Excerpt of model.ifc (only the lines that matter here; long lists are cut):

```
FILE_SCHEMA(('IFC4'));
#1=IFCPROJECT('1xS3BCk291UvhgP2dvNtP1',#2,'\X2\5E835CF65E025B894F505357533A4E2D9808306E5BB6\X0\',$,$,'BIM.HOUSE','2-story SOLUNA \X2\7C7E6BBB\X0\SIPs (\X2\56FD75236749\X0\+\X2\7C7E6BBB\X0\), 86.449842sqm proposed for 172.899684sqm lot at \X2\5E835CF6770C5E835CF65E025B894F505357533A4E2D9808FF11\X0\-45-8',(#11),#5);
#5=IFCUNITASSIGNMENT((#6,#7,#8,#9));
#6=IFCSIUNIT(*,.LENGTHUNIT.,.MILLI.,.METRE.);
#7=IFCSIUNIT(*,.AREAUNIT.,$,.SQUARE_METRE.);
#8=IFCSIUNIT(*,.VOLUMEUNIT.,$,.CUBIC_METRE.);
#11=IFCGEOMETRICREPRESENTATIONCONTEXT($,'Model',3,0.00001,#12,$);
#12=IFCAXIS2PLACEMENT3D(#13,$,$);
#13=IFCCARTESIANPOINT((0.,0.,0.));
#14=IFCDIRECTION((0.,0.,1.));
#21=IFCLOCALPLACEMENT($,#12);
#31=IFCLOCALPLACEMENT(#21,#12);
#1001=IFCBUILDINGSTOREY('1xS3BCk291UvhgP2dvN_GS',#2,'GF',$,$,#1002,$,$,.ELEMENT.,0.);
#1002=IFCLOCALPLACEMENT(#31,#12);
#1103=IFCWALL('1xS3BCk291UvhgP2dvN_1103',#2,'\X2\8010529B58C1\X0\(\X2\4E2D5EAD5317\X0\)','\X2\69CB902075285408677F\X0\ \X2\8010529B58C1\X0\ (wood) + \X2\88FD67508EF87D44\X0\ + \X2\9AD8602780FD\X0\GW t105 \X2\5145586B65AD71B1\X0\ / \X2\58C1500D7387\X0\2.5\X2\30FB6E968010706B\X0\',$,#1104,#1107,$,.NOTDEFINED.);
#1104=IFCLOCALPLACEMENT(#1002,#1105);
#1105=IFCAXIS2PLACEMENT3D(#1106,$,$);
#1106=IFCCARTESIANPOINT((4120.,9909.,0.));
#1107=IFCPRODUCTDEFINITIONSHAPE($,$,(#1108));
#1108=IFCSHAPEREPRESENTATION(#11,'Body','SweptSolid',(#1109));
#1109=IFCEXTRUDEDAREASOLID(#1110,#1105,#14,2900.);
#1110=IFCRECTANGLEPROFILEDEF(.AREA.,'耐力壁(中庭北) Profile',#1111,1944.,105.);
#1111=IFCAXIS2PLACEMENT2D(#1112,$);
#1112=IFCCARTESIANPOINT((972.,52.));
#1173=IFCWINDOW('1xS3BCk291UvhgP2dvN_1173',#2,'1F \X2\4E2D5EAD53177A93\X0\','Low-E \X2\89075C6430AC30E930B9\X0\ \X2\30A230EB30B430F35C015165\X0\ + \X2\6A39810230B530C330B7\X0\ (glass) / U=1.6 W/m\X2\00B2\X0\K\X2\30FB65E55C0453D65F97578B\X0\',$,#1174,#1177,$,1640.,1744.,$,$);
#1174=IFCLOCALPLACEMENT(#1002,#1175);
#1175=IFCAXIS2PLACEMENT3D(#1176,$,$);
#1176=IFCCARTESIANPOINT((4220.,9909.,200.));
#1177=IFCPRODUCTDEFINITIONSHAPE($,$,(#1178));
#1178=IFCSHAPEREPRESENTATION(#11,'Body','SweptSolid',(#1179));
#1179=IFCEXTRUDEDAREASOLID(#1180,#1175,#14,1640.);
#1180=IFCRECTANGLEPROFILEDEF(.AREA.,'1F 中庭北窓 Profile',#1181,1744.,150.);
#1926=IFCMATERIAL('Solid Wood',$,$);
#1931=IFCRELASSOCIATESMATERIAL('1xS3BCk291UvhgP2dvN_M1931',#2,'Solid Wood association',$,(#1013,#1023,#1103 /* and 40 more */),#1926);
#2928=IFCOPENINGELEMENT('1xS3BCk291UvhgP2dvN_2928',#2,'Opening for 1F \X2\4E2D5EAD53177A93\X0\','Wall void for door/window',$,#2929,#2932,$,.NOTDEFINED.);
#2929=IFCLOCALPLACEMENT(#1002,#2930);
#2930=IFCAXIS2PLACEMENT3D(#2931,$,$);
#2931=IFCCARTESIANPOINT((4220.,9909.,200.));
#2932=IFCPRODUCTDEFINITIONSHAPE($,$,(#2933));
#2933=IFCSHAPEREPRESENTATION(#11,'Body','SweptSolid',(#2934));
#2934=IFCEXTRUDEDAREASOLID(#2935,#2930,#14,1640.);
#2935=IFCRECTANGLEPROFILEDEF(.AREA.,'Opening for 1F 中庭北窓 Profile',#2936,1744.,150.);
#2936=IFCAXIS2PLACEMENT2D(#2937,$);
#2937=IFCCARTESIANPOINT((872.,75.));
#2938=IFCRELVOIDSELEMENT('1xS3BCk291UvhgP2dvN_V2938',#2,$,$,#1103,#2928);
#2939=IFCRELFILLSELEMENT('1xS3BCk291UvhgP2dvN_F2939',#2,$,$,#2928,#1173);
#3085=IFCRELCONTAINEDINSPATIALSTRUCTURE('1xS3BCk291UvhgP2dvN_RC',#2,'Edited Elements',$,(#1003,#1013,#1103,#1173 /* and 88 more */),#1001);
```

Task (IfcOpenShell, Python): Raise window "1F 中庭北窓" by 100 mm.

```python
import numpy as np
import ifcopenshell
import ifcopenshell.api.geometry
import ifcopenshell.util.placement
import ifcopenshell.util.unit

model = ifcopenshell.open("model.ifc")
unit_scale = ifcopenshell.util.unit.calculate_unit_scale(model)

window = model.by_guid("1xS3BCk291UvhgP2dvN_1173")
opening = window.FillsVoids[0].RelatingOpeningElement
dz = 0.1 / unit_scale

shift = np.array([0.0, 0.0, dz])
# The window is not placed relative to its opening, so move both.
for product in (opening, window):
    matrix = ifcopenshell.util.placement.get_local_placement(product.ObjectPlacement)
    matrix[:3, 3] += shift
    ifcopenshell.api.geometry.edit_object_placement(model, product=product, matrix=matrix, is_si=False)

print(f"moved by {dz * unit_scale:+.3f} m")

model.write("model-out.ifc")
```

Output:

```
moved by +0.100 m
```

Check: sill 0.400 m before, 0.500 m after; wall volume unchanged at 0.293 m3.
